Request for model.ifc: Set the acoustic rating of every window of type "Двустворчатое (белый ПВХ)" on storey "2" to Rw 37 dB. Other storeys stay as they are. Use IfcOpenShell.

First a look at what the model holds.

```python
import ifcopenshell
import ifcopenshell.util.element

model = ifcopenshell.open("model.ifc")
print(model.schema)
storey = next(s for s in model.by_type("IfcBuildingStorey") if s.Name == "2")
windows = [e for e in ifcopenshell.util.element.get_decomposition(storey) if e.is_a("IfcWindow")]
seen = {}
for e in windows:
    element_type = ifcopenshell.util.element.get_type(e)
    key = (element_type.Name if element_type != e and element_type else None, ifcopenshell.util.element.get_pset(e, "Pset_WindowCommon", "AcousticRating"))
    seen[key] = seen.get(key, 0) + 1
for (name, value), count in sorted(seen.items(), key=str):
    print(count, "x", name, "|", value)
```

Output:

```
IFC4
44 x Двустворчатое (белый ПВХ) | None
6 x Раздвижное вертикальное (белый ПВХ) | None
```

```python
import ifcopenshell
import ifcopenshell.api.pset
import ifcopenshell.util.element

model = ifcopenshell.open("model.ifc")

storey = next(s for s in model.by_type("IfcBuildingStorey") if s.Name == "2")
windows = [e for e in ifcopenshell.util.element.get_decomposition(storey) if e.is_a("IfcWindow")]

count = 0
for e in windows:
    element_type = ifcopenshell.util.element.get_type(e)
    if element_type in (None, e) or element_type.Name != "Двустворчатое (белый ПВХ)":
        continue
    # add_pset returns the element's existing set when there is one.
    pset = ifcopenshell.api.pset.add_pset(model, product=e, name="Pset_WindowCommon")
    ifcopenshell.api.pset.edit_pset(model, pset=pset, properties={"AcousticRating": "Rw 37 dB"})
    count += 1

print(count, "windows updated")

model.write("model-out.ifc")
```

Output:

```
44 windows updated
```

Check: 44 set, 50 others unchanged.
